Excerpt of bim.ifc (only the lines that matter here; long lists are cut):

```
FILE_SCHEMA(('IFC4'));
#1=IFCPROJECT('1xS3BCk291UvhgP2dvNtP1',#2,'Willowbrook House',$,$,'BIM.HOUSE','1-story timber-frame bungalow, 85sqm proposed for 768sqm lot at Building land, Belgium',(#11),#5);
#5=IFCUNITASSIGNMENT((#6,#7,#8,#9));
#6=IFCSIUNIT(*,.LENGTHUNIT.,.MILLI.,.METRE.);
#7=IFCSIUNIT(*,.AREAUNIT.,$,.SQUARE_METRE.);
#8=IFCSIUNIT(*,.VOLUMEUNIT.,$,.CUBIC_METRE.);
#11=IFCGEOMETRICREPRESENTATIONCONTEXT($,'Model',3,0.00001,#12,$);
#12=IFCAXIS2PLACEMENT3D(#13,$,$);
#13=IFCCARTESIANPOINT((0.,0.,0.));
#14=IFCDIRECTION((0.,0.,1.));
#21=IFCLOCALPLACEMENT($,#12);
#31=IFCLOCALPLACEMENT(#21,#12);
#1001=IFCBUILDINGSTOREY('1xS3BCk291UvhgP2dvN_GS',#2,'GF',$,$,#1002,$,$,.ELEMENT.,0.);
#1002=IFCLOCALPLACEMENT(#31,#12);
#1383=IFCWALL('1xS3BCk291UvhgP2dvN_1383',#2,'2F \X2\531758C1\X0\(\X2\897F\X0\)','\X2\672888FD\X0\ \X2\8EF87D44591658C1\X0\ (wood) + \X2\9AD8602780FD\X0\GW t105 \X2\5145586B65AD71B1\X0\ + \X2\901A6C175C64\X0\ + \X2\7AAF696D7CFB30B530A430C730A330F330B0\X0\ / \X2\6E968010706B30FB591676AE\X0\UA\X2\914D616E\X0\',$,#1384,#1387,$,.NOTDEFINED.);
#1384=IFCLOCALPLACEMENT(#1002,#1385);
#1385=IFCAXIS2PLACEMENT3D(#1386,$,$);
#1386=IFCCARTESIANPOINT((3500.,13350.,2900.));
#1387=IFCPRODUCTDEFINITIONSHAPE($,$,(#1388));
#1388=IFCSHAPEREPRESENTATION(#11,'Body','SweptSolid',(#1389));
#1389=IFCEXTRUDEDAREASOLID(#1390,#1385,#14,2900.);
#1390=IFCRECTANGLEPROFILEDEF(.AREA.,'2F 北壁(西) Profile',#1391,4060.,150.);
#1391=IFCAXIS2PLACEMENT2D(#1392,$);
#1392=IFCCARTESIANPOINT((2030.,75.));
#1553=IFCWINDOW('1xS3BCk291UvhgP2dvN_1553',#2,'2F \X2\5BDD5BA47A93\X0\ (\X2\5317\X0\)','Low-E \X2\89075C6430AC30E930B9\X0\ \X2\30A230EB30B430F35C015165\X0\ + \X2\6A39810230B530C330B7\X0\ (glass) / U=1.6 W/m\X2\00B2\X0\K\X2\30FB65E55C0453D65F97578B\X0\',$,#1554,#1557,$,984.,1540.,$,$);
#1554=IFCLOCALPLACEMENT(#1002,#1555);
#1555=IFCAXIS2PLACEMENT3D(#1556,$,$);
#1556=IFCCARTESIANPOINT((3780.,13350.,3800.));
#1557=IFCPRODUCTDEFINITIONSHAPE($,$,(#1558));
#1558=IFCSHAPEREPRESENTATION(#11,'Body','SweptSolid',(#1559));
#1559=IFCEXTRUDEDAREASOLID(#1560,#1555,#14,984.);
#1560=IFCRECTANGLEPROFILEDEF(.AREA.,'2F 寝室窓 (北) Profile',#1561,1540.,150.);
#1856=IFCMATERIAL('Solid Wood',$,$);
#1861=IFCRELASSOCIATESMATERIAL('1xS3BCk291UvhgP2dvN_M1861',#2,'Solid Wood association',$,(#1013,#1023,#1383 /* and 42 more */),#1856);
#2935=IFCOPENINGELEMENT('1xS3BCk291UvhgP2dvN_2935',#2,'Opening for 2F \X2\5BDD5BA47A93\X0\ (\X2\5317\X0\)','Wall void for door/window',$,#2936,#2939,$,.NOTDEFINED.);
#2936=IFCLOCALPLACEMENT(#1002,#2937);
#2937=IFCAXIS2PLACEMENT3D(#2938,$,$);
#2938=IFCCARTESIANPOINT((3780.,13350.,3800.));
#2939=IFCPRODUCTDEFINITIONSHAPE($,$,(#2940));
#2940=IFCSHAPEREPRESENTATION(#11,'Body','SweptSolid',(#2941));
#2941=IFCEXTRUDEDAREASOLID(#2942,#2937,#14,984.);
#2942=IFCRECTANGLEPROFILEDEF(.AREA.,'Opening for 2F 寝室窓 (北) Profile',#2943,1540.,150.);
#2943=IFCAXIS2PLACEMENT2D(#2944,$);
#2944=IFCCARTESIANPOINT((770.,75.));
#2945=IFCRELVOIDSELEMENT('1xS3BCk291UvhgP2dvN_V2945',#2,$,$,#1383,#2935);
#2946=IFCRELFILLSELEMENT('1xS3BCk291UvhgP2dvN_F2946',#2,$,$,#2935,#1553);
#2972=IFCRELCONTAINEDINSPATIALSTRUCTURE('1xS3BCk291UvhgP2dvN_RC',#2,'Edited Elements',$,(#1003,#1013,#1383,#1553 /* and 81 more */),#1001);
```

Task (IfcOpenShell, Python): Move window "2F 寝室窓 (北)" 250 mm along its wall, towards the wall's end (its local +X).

```python
import ifcopenshell
import ifcopenshell.api.geometry
import ifcopenshell.util.placement
import ifcopenshell.util.unit

model = ifcopenshell.open("bim.ifc")
unit_scale = ifcopenshell.util.unit.calculate_unit_scale(model)

window = model.by_guid("1xS3BCk291UvhgP2dvN_1553")
opening = window.FillsVoids[0].RelatingOpeningElement
wall = opening.VoidsElements[0].RelatingBuildingElement

wall_matrix = ifcopenshell.util.placement.get_local_placement(wall.ObjectPlacement)
shift = wall_matrix[:3, 0] * 0.25 / unit_scale
before = ifcopenshell.util.placement.get_local_placement(window.ObjectPlacement)[:3, 3].copy()

# The window is not placed relative to its opening, so move both.
for product in (opening, window):
    matrix = ifcopenshell.util.placement.get_local_placement(product.ObjectPlacement)
    matrix[:3, 3] += shift
    ifcopenshell.api.geometry.edit_object_placement(model, product=product, matrix=matrix, is_si=False)

after = ifcopenshell.util.placement.get_local_placement(window.ObjectPlacement)[:3, 3]
print("window moved by", (after - before).round(3) + 0.0)

model.write("bim-out.ifc")
```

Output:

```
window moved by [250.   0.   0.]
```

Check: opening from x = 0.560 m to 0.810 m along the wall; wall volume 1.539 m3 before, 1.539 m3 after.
